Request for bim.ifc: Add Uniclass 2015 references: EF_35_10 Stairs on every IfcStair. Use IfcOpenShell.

First a look at what the model holds.

```python
import ifcopenshell

model = ifcopenshell.open("bim.ifc")
print(model.schema)
print("classifications:", [c.Name for c in model.by_type("IfcClassification")])
for ifc_class in ("IfcDoor", "IfcRoof", "IfcStair", "IfcWall", "IfcWindow"):
    print(ifc_class, len(model.by_type(ifc_class)))
```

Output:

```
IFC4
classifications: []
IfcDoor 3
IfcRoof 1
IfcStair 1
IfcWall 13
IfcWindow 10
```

```python
import ifcopenshell
import ifcopenshell.api.classification

model = ifcopenshell.open("bim.ifc")

system = ifcopenshell.api.classification.add_classification(model, classification="Uniclass 2015")

codes = {
    "IfcStair": ("EF_35_10", "Stairs"),
}
for ifc_class, (code, name) in codes.items():
    products = model.by_type(ifc_class)
    ifcopenshell.api.classification.add_reference(
        model, products=products, classification=system, identification=code, name=name
    )
    print(code, len(products))

model.write("bim_updated.ifc")
```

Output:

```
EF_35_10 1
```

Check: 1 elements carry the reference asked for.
